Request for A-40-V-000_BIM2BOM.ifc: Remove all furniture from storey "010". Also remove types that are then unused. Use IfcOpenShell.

First a look at what the model holds.

```python
import ifcopenshell
import ifcopenshell.util.element

model = ifcopenshell.open("A-40-V-000_BIM2BOM.ifc")
print(model.schema)
storey = next(s for s in model.by_type("IfcBuildingStorey") if s.Name == "010")
furniture = [e for e in ifcopenshell.util.element.get_decomposition(storey) if e.is_a("IfcFurnishingElement")]
seen = {}
for e in furniture:
    element_type = ifcopenshell.util.element.get_type(e)
    name = element_type.Name if element_type not in (None, e) else None
    seen[name] = seen.get(name, 0) + 1
for name, count in sorted(seen.items(), key=str):
    print(count, "x", name)
```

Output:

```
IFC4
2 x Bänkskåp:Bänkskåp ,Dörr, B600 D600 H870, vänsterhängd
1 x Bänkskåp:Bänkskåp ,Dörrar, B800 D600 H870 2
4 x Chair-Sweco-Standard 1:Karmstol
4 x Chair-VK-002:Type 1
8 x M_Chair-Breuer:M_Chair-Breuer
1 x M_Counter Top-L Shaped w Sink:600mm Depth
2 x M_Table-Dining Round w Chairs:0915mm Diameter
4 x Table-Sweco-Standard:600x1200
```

```python
import ifcopenshell
import ifcopenshell.api.root
import ifcopenshell.util.element

model = ifcopenshell.open("A-40-V-000_BIM2BOM.ifc")

storey = next(s for s in model.by_type("IfcBuildingStorey") if s.Name == "010")
furniture = [e for e in ifcopenshell.util.element.get_decomposition(storey) if e.is_a("IfcFurnishingElement")]
types = {ifcopenshell.util.element.get_type(e) for e in furniture} - {None, *furniture}

for e in furniture:
    ifcopenshell.api.root.remove_product(model, product=e)
print(len(furniture), "removed")

unused = [t for t in types if not ifcopenshell.util.element.get_types(t)]
for t in unused:
    ifcopenshell.api.root.remove_product(model, product=t)
print(len(unused), "unused types removed")

model.write("A-40-V-000_BIM2BOM_rev.ifc")
```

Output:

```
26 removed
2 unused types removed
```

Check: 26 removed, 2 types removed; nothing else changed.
